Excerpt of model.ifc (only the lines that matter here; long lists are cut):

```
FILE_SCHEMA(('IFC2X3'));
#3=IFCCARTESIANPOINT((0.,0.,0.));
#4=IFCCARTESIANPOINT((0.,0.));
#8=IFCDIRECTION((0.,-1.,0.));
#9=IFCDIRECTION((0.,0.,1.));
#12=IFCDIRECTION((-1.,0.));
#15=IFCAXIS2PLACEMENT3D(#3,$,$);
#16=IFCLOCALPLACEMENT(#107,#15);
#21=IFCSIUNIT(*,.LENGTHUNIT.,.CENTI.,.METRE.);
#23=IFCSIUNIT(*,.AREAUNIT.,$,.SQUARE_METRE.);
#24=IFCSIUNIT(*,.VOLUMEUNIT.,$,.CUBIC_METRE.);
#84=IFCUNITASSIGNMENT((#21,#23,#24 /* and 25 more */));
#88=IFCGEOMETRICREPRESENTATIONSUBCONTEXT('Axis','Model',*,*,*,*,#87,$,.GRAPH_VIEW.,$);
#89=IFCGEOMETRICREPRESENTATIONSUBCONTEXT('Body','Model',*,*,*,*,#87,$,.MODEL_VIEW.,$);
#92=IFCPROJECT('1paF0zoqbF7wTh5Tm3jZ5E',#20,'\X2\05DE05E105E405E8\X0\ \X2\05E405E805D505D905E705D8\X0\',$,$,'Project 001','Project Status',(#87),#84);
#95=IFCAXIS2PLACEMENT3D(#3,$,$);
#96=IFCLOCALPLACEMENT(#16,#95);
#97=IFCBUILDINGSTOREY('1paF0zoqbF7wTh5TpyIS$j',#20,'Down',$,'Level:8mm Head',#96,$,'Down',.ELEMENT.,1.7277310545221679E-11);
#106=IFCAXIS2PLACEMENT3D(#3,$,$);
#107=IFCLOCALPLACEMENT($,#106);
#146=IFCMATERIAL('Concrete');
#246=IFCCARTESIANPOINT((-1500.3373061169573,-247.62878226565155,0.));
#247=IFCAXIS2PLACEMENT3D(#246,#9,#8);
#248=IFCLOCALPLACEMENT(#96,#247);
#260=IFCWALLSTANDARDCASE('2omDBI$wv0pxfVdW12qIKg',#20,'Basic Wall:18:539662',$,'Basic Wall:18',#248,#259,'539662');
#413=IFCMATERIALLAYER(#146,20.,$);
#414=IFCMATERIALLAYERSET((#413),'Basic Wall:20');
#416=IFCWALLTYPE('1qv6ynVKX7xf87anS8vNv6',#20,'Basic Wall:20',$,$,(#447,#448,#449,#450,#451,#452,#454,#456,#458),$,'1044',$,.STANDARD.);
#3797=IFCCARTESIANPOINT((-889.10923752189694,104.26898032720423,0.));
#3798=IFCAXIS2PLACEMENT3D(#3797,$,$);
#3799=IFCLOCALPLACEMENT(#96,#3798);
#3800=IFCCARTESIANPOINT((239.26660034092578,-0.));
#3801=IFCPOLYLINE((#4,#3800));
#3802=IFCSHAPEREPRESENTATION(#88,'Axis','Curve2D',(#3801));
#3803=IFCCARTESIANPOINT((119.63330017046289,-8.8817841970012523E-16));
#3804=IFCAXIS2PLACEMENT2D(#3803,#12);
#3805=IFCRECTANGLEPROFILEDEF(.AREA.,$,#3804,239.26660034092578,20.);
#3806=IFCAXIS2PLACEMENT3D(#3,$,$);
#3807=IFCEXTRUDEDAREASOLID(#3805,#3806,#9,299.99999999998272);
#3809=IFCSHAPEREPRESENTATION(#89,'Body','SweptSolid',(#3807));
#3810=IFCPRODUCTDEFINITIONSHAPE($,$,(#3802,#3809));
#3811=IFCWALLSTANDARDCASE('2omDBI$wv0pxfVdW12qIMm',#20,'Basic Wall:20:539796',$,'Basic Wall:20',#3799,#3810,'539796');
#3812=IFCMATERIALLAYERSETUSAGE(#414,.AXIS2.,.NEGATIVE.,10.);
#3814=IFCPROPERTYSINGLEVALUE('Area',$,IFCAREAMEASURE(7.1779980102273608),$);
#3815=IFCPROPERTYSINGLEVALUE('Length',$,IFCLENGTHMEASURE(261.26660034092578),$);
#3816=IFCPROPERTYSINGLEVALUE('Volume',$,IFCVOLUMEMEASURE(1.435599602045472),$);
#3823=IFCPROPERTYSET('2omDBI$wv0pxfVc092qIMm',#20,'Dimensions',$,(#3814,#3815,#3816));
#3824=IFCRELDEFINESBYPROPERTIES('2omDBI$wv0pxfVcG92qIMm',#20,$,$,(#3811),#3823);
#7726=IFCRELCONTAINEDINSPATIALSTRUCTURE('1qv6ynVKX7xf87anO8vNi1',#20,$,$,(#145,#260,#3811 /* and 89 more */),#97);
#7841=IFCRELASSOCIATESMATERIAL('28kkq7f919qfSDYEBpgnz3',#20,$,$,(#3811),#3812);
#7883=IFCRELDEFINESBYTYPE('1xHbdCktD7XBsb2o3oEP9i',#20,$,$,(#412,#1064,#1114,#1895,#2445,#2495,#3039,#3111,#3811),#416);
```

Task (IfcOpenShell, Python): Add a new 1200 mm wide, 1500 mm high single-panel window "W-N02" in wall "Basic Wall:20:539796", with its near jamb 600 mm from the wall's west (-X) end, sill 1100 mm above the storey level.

```python
import numpy as np
import ifcopenshell
import ifcopenshell.api.feature
import ifcopenshell.api.geometry
import ifcopenshell.api.pset
import ifcopenshell.api.root
import ifcopenshell.api.spatial
import ifcopenshell.api.type
import ifcopenshell.geom
import ifcopenshell.util.element
import ifcopenshell.util.placement
import ifcopenshell.util.representation
import ifcopenshell.util.shape
import ifcopenshell.util.unit

model = ifcopenshell.open("model.ifc")
unit_scale = ifcopenshell.util.unit.calculate_unit_scale(model)
area_scale = ifcopenshell.util.unit.calculate_unit_scale(model, "AREAUNIT")
volume_scale = ifcopenshell.util.unit.calculate_unit_scale(model, "VOLUMEUNIT")
settings = ifcopenshell.geom.settings()


def volume(element):
    """Net volume in cubic metres, openings subtracted."""
    shape = ifcopenshell.geom.create_shape(settings, element)
    return ifcopenshell.util.shape.get_volume(shape.geometry)


wall = model.by_guid("2omDBI$wv0pxfVdW12qIMm")
storey = ifcopenshell.util.element.get_container(wall, ifc_class="IfcBuildingStorey")
context = ifcopenshell.util.representation.get_context(model, "Model", "Body", "MODEL_VIEW")
before = volume(wall)

width, height, from_end, sill = 1.2, 1.5, 0.6, 1.1  # metres

# The wall runs along its own X axis, and the end named is its -X end.
wall_shape = ifcopenshell.geom.create_shape(settings, wall)
x, y, z = ifcopenshell.util.shape.get_vertices(wall_shape.geometry).T
start = x.min() + from_end
face, thickness = float(y.min()), float(y.max() - y.min())
wall_matrix = ifcopenshell.util.placement.get_local_placement(wall.ObjectPlacement)
level = ifcopenshell.util.placement.get_local_placement(storey.ObjectPlacement)[2, 3]


def in_wall(x, y):
    """Placement at x, y metres in the wall's axes, at sill height."""
    matrix = wall_matrix.copy()
    matrix[:, 3] = wall_matrix @ np.array([x / unit_scale, y / unit_scale, 0.0, 1.0])
    matrix[2, 3] = level + sill / unit_scale
    return matrix


# Opening: a box that overshoots both wall faces by 50 mm.
opening = ifcopenshell.api.root.create_entity(model, ifc_class="IfcOpeningElement")
box = ifcopenshell.api.geometry.add_wall_representation(
    model, context=context, length=width, height=height, thickness=thickness + 0.1
)
ifcopenshell.api.geometry.assign_representation(model, product=opening, representation=box)
ifcopenshell.api.geometry.edit_object_placement(model, product=opening, matrix=in_wall(start, face - 0.05), is_si=False)
ifcopenshell.api.feature.add_feature(model, feature=opening, element=wall)

window = ifcopenshell.api.root.create_entity(model, ifc_class="IfcWindow", name="W-N02")
window.OverallWidth, window.OverallHeight = width / unit_scale, height / unit_scale
body = ifcopenshell.api.geometry.add_window_representation(
    model,
    context=context,
    overall_width=window.OverallWidth,
    overall_height=window.OverallHeight,
    partition_type="SINGLE_PANEL",
)
ifcopenshell.api.geometry.assign_representation(model, product=window, representation=body)
ifcopenshell.api.spatial.assign_container(model, products=[window], relating_structure=storey)
fills = ifcopenshell.api.feature.add_filling(model, opening=opening, element=window)
fills.OwnerHistory = window.OwnerHistory  # required in IFC2X3

# IFC2X3 keeps the operation on the window style.
style = ifcopenshell.api.root.create_entity(model, ifc_class="IfcWindowStyle", name="W-N02")
style.OperationType, style.ConstructionType = "SINGLE_PANEL", "NOTDEFINED"
style.ParameterTakesPrecedence = style.Sizeable = False
ifcopenshell.api.type.assign_type(model, related_objects=[window], relating_type=style)

# Centre the window in the wall's thickness.
ifcopenshell.api.geometry.edit_object_placement(model, product=window, matrix=in_wall(start, face), is_si=False)
window_shape = ifcopenshell.geom.create_shape(settings, window)
depth = ifcopenshell.util.shape.get_vertices(window_shape.geometry)[:, 1]
offset = face + thickness / 2 - (depth.min() + depth.max()) / 2
ifcopenshell.api.geometry.edit_object_placement(model, product=window, matrix=in_wall(start, offset), is_si=False)

after = volume(wall)

# Update the wall's stored quantities.
pset = model.by_id(ifcopenshell.util.element.get_pset(wall, "Dimensions", should_inherit=False)["id"])
ifcopenshell.api.pset.edit_pset(model, pset=pset, properties={
    "Area": model.create_entity("IfcAreaMeasure", after / thickness / area_scale),
    "Volume": model.create_entity("IfcVolumeMeasure", after / volume_scale),
})

print(f"wall volume {before:.3f} -> {after:.3f} m3")

model.write("model_v2.ifc")
```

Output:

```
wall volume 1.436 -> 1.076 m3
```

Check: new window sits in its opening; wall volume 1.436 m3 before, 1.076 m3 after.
